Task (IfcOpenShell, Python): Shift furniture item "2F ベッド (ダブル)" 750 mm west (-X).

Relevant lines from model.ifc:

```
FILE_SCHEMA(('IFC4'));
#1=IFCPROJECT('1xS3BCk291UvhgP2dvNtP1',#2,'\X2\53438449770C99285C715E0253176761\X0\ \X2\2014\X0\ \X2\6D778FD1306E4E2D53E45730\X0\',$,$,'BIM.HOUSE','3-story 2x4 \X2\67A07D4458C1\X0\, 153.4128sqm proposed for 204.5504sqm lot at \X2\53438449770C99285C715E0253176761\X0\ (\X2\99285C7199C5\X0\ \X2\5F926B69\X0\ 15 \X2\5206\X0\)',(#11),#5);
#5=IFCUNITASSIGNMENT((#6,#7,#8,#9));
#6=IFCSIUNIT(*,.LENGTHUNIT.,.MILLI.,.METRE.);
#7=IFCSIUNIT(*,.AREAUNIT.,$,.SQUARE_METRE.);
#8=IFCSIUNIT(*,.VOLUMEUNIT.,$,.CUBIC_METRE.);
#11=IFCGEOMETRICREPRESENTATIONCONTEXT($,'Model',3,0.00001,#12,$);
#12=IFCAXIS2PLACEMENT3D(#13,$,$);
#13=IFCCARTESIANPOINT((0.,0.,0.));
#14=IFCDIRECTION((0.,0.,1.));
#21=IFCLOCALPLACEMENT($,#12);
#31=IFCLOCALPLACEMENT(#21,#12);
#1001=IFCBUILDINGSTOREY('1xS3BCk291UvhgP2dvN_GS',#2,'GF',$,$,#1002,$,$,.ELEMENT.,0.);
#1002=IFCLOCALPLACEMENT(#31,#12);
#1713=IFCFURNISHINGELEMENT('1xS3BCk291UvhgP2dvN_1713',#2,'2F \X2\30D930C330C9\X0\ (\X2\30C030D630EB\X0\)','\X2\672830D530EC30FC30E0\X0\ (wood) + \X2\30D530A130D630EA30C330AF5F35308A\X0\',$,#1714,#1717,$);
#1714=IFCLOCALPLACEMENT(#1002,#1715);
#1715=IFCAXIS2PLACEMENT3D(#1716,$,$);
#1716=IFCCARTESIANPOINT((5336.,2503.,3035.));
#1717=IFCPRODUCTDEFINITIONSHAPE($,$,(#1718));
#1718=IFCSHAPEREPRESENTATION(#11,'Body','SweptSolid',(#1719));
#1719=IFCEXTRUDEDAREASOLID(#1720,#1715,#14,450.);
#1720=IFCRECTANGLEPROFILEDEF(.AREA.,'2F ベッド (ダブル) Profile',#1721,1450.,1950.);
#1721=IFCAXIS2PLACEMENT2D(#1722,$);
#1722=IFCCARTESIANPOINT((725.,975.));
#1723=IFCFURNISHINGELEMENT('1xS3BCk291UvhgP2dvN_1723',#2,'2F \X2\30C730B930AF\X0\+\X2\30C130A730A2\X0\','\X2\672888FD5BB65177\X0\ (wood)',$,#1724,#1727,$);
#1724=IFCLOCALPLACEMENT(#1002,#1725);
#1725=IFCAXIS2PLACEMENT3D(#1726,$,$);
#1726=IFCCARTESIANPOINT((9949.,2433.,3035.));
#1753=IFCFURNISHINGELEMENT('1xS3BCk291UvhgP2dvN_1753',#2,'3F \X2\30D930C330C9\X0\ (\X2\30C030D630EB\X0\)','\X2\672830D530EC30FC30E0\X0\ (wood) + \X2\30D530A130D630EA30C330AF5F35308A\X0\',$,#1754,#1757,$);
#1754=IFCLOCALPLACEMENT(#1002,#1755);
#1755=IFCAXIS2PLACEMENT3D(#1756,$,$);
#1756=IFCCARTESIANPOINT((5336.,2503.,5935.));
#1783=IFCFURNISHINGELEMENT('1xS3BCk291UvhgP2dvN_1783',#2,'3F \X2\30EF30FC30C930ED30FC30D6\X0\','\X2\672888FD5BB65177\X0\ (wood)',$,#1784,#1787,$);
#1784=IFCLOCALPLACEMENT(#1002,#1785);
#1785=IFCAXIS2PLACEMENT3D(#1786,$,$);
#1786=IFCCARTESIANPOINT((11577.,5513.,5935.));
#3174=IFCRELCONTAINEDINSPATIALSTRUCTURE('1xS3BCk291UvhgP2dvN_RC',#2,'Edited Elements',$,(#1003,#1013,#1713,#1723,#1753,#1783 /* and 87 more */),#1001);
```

```python
import ifcopenshell
import ifcopenshell.api.geometry
import ifcopenshell.util.placement

model = ifcopenshell.open("model.ifc")

item = model.by_guid("1xS3BCk291UvhgP2dvN_1713")
matrix = ifcopenshell.util.placement.get_local_placement(item.ObjectPlacement)
matrix[0, 3] -= 750.0
ifcopenshell.api.geometry.edit_object_placement(model, product=item, matrix=matrix, is_si=False)

print(ifcopenshell.util.placement.get_local_placement(item.ObjectPlacement).round(3) + 0.0)

model.write("model_updated.ifc")
```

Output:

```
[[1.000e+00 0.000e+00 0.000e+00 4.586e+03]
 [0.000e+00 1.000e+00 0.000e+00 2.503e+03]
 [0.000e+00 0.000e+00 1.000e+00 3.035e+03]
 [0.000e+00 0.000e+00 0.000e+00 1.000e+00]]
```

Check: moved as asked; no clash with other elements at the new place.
